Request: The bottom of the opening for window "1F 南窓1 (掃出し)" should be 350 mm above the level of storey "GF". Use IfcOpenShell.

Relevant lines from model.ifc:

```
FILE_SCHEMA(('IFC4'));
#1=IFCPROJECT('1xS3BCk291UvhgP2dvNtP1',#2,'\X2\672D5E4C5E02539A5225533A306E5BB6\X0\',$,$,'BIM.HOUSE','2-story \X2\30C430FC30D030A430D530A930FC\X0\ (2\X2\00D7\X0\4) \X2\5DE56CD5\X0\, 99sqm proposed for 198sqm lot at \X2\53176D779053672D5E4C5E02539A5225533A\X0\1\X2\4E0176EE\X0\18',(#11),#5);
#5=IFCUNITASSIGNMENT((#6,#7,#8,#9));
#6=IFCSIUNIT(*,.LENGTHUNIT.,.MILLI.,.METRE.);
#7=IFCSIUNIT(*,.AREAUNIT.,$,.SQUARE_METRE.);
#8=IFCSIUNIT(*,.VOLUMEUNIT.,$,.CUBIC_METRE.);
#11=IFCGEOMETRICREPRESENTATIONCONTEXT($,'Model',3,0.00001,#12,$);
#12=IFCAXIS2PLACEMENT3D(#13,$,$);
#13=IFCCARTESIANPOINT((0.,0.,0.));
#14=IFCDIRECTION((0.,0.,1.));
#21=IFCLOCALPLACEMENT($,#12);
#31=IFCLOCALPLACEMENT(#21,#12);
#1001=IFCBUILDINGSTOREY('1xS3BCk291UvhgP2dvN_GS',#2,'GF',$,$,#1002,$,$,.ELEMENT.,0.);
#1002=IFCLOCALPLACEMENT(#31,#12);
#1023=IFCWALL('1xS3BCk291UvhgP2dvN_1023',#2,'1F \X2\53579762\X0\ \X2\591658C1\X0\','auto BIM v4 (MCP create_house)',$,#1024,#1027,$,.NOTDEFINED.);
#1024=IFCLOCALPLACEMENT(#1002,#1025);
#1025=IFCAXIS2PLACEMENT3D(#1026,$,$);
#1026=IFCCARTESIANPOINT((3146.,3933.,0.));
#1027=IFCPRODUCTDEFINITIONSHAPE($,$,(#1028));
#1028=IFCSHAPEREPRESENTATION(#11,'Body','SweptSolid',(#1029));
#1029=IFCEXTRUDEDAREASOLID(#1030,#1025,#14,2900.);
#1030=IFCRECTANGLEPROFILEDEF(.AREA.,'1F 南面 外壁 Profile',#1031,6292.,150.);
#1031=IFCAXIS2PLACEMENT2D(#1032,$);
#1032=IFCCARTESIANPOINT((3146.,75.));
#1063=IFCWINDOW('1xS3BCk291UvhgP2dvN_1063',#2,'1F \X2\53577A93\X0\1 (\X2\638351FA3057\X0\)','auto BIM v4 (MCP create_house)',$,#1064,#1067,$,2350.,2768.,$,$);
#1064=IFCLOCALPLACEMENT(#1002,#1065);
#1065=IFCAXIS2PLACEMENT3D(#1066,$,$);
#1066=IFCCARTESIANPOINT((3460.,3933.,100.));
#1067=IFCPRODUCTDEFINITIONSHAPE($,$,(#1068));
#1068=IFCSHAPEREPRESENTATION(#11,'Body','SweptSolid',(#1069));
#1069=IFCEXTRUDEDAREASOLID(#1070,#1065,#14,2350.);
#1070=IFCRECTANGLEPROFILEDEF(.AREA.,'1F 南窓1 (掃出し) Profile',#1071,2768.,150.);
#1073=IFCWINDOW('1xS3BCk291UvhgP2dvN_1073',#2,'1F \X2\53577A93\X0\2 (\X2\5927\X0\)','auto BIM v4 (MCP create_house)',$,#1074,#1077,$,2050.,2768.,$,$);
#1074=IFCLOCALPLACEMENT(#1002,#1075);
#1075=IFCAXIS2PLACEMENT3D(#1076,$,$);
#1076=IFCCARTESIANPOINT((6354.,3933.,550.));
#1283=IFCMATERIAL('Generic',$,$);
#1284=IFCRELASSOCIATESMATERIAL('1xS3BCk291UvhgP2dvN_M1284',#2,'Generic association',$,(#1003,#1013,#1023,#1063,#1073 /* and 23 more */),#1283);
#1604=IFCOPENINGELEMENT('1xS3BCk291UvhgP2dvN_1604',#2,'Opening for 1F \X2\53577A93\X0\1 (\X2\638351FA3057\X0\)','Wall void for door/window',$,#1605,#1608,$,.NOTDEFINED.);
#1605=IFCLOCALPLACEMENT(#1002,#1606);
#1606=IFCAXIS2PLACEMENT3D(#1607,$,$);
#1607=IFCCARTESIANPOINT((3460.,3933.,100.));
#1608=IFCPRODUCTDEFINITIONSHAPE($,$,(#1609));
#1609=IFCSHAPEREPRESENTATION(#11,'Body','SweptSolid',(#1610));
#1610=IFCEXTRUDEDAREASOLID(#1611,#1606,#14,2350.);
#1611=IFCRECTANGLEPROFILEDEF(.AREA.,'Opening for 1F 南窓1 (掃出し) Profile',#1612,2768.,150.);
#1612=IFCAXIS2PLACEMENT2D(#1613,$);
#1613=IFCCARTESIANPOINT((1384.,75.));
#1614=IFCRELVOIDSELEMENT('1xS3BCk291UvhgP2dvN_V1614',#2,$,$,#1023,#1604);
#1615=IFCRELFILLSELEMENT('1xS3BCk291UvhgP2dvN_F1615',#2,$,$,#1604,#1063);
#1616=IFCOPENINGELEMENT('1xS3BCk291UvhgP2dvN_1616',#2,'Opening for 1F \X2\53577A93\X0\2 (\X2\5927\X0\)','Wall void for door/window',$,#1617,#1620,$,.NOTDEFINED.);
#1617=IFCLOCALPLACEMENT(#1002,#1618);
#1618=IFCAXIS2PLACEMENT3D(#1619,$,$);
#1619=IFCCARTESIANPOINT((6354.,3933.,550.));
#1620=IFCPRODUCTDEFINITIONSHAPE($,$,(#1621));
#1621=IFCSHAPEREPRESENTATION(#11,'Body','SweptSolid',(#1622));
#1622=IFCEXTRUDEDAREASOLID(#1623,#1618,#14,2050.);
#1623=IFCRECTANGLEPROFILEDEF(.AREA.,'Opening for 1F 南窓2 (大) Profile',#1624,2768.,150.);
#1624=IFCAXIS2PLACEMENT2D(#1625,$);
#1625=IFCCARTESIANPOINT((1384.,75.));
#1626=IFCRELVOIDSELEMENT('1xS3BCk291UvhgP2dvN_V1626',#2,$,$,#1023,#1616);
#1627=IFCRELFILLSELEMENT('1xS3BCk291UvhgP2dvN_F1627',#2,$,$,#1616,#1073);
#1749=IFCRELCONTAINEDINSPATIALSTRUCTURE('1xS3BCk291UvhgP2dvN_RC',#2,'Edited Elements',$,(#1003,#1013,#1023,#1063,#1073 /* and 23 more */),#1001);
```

```python
import numpy as np
import ifcopenshell
import ifcopenshell.api.geometry
import ifcopenshell.geom
import ifcopenshell.util.element
import ifcopenshell.util.placement
import ifcopenshell.util.shape
import ifcopenshell.util.unit

model = ifcopenshell.open("model.ifc")
unit_scale = ifcopenshell.util.unit.calculate_unit_scale(model)

window = model.by_guid("1xS3BCk291UvhgP2dvN_1063")
opening = window.FillsVoids[0].RelatingOpeningElement
storey = ifcopenshell.util.element.get_container(window, ifc_class="IfcBuildingStorey")
level = ifcopenshell.util.placement.get_local_placement(storey.ObjectPlacement)[2, 3]

# The opening's origin need not be at the sill, so measure its lowest point.
shape = ifcopenshell.geom.create_shape(ifcopenshell.geom.settings(), opening)
bottom = ifcopenshell.util.shape.get_shape_bottom_elevation(shape, shape.geometry) / unit_scale
dz = level + 350.0 - bottom

shift = np.array([0.0, 0.0, dz])
# The window is not placed relative to its opening, so move both.
for product in (opening, window):
    matrix = ifcopenshell.util.placement.get_local_placement(product.ObjectPlacement)
    matrix[:3, 3] += shift
    ifcopenshell.api.geometry.edit_object_placement(model, product=product, matrix=matrix, is_si=False)

print(f"moved by {dz * unit_scale:+.3f} m")

model.write("model_updated.ifc")
```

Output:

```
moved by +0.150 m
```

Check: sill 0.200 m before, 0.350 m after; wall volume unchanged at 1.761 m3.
